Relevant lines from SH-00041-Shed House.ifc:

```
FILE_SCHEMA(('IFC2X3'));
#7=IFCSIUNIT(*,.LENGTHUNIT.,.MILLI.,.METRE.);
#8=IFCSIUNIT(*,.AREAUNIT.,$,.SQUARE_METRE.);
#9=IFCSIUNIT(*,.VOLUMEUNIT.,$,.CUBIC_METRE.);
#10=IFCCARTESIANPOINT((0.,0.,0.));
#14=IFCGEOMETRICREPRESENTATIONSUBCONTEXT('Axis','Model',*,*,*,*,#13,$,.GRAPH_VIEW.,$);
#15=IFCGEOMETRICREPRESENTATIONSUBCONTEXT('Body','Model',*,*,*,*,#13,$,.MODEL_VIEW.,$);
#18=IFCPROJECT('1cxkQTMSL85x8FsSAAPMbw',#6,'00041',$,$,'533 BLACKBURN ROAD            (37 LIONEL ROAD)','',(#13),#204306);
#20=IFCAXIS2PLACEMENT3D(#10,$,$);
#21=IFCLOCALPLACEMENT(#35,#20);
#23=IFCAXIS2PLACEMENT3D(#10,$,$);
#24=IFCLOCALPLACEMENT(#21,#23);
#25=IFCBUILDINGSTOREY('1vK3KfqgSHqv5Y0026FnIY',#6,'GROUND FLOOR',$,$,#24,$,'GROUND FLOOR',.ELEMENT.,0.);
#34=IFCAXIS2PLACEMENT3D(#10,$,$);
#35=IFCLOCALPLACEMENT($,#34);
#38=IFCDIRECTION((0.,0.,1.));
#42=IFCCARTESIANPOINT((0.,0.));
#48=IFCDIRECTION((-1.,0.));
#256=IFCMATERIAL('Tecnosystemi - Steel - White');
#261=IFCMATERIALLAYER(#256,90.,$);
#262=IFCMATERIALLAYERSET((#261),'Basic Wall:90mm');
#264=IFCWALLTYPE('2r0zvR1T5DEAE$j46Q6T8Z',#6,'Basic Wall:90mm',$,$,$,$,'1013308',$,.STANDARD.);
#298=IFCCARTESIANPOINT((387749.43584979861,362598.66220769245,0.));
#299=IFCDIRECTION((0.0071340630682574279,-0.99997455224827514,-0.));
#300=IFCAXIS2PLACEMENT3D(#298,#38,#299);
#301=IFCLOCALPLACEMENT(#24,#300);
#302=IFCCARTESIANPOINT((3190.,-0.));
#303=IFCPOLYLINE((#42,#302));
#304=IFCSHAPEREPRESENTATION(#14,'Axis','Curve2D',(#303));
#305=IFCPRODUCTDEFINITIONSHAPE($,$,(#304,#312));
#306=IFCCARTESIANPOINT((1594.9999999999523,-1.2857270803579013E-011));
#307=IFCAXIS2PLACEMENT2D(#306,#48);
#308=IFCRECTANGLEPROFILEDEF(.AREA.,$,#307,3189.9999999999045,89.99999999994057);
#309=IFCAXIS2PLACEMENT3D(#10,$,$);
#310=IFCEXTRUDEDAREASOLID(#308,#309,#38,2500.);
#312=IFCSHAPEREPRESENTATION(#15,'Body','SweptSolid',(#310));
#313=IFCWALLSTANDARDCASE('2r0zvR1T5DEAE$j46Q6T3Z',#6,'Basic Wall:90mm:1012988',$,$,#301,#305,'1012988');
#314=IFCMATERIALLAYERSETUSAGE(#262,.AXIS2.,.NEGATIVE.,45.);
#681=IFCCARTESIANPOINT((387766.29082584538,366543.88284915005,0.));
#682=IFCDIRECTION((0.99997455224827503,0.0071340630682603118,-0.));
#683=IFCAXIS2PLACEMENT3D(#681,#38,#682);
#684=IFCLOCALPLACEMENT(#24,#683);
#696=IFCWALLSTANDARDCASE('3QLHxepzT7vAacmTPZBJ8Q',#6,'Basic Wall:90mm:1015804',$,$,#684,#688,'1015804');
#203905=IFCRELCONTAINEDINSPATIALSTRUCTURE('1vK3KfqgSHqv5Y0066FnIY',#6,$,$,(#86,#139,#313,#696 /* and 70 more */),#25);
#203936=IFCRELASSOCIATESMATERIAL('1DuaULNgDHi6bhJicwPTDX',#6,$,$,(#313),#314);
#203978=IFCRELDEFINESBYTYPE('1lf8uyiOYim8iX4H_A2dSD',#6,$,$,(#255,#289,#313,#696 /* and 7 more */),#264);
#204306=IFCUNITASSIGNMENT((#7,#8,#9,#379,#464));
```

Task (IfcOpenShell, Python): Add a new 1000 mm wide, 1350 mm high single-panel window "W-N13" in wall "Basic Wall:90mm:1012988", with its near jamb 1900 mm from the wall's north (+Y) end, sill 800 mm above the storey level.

```python
import numpy as np
import ifcopenshell
import ifcopenshell.api.feature
import ifcopenshell.api.geometry
import ifcopenshell.api.root
import ifcopenshell.api.spatial
import ifcopenshell.api.type
import ifcopenshell.geom
import ifcopenshell.util.element
import ifcopenshell.util.placement
import ifcopenshell.util.representation
import ifcopenshell.util.shape
import ifcopenshell.util.unit

model = ifcopenshell.open("SH-00041-Shed House.ifc")
unit_scale = ifcopenshell.util.unit.calculate_unit_scale(model)
settings = ifcopenshell.geom.settings()


def volume(element):
    """Net volume in cubic metres, openings subtracted."""
    shape = ifcopenshell.geom.create_shape(settings, element)
    return ifcopenshell.util.shape.get_volume(shape.geometry)


wall = model.by_guid("2r0zvR1T5DEAE$j46Q6T3Z")
storey = ifcopenshell.util.element.get_container(wall, ifc_class="IfcBuildingStorey")
context = ifcopenshell.util.representation.get_context(model, "Model", "Body", "MODEL_VIEW")
before = volume(wall)

width, height, from_end, sill = 1, 1.35, 1.9, 0.8  # metres

# The wall runs along its own X axis, and the end named is its -X end.
wall_shape = ifcopenshell.geom.create_shape(settings, wall)
x, y, z = ifcopenshell.util.shape.get_vertices(wall_shape.geometry).T
start = x.min() + from_end
face, thickness = float(y.min()), float(y.max() - y.min())
wall_matrix = ifcopenshell.util.placement.get_local_placement(wall.ObjectPlacement)
level = ifcopenshell.util.placement.get_local_placement(storey.ObjectPlacement)[2, 3]


def in_wall(x, y):
    """Placement at x, y metres in the wall's axes, at sill height."""
    matrix = wall_matrix.copy()
    matrix[:, 3] = wall_matrix @ np.array([x / unit_scale, y / unit_scale, 0.0, 1.0])
    matrix[2, 3] = level + sill / unit_scale
    return matrix


# Opening: a box that overshoots both wall faces by 50 mm.
opening = ifcopenshell.api.root.create_entity(model, ifc_class="IfcOpeningElement")
box = ifcopenshell.api.geometry.add_wall_representation(
    model, context=context, length=width, height=height, thickness=thickness + 0.1
)
ifcopenshell.api.geometry.assign_representation(model, product=opening, representation=box)
ifcopenshell.api.geometry.edit_object_placement(model, product=opening, matrix=in_wall(start, face - 0.05), is_si=False)
ifcopenshell.api.feature.add_feature(model, feature=opening, element=wall)

window = ifcopenshell.api.root.create_entity(model, ifc_class="IfcWindow", name="W-N13")
window.OverallWidth, window.OverallHeight = width / unit_scale, height / unit_scale
body = ifcopenshell.api.geometry.add_window_representation(
    model,
    context=context,
    overall_width=window.OverallWidth,
    overall_height=window.OverallHeight,
    partition_type="SINGLE_PANEL",
)
ifcopenshell.api.geometry.assign_representation(model, product=window, representation=body)
ifcopenshell.api.spatial.assign_container(model, products=[window], relating_structure=storey)
fills = ifcopenshell.api.feature.add_filling(model, opening=opening, element=window)
fills.OwnerHistory = window.OwnerHistory  # required in IFC2X3

# IFC2X3 keeps the operation on the window style.
style = ifcopenshell.api.root.create_entity(model, ifc_class="IfcWindowStyle", name="W-N13")
style.OperationType, style.ConstructionType = "SINGLE_PANEL", "NOTDEFINED"
style.ParameterTakesPrecedence = style.Sizeable = False
ifcopenshell.api.type.assign_type(model, related_objects=[window], relating_type=style)

# Centre the window in the wall's thickness.
ifcopenshell.api.geometry.edit_object_placement(model, product=window, matrix=in_wall(start, face), is_si=False)
window_shape = ifcopenshell.geom.create_shape(settings, window)
depth = ifcopenshell.util.shape.get_vertices(window_shape.geometry)[:, 1]
offset = face + thickness / 2 - (depth.min() + depth.max()) / 2
ifcopenshell.api.geometry.edit_object_placement(model, product=window, matrix=in_wall(start, offset), is_si=False)

after = volume(wall)

print(f"wall volume {before:.3f} -> {after:.3f} m3")

model.write("SH-00041-Shed House_rev.ifc")
```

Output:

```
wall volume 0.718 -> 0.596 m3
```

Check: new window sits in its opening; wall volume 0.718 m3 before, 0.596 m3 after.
